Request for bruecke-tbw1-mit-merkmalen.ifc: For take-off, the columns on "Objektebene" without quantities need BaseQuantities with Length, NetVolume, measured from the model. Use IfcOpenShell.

First a look at what the model holds.

```python
import ifcopenshell
import ifcopenshell.util.element
import ifcopenshell.util.unit

model = ifcopenshell.open("bruecke-tbw1-mit-merkmalen.ifc")
print(model.schema)
for unit_type in ("LENGTHUNIT", "AREAUNIT", "VOLUMEUNIT"):
    print(unit_type, ifcopenshell.util.unit.calculate_unit_scale(model, unit_type))
storey = next(s for s in model.by_type("IfcBuildingStorey") if s.Name == "Objektebene")
columns = [e for e in ifcopenshell.util.element.get_decomposition(storey) if e.is_a("IfcColumn")]
for e in sorted(columns, key=lambda e: e.id()):
    print(e.id(), e.is_a(), e.Name, list(ifcopenshell.util.element.get_psets(e, qtos_only=True)), sep=" | ")
```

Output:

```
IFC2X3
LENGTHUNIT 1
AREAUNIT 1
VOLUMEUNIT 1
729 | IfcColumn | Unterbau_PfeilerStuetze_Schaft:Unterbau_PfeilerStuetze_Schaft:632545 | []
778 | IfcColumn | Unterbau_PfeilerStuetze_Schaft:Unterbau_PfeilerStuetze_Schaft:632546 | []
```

```python
import ifcopenshell
import ifcopenshell.api.pset
import ifcopenshell.geom
import ifcopenshell.util.element
import ifcopenshell.util.shape
import ifcopenshell.util.unit

model = ifcopenshell.open("bruecke-tbw1-mit-merkmalen.ifc")
unit_scale = ifcopenshell.util.unit.calculate_unit_scale(model)
volume_scale = ifcopenshell.util.unit.calculate_unit_scale(model, "VOLUMEUNIT")
settings = ifcopenshell.geom.settings()

storey = next(s for s in model.by_type("IfcBuildingStorey") if s.Name == "Objektebene")
columns = [e for e in ifcopenshell.util.element.get_decomposition(storey) if e.is_a("IfcColumn")]

for e in sorted(columns, key=lambda e: e.id()):
    if ifcopenshell.util.element.get_psets(e, qtos_only=True, should_inherit=False):
        continue
    # Geometry comes back in metres, in the element's own axes.
    shape = ifcopenshell.geom.create_shape(settings, e)
    values = {
        "Length": ifcopenshell.util.shape.get_z(shape.geometry) / unit_scale,
        "NetVolume": ifcopenshell.util.shape.get_volume(shape.geometry) / volume_scale,
    }
    qto = ifcopenshell.api.pset.add_qto(model, product=e, name="BaseQuantities")
    ifcopenshell.api.pset.edit_qto(model, qto=qto, properties=values)
    print(e.id(), {k: round(v, 3) for k, v in values.items()})

model.write("bruecke-tbw1-mit-merkmalen-out.ifc")
```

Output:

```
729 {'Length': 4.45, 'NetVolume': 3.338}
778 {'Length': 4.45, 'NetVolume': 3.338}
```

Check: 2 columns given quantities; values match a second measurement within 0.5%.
